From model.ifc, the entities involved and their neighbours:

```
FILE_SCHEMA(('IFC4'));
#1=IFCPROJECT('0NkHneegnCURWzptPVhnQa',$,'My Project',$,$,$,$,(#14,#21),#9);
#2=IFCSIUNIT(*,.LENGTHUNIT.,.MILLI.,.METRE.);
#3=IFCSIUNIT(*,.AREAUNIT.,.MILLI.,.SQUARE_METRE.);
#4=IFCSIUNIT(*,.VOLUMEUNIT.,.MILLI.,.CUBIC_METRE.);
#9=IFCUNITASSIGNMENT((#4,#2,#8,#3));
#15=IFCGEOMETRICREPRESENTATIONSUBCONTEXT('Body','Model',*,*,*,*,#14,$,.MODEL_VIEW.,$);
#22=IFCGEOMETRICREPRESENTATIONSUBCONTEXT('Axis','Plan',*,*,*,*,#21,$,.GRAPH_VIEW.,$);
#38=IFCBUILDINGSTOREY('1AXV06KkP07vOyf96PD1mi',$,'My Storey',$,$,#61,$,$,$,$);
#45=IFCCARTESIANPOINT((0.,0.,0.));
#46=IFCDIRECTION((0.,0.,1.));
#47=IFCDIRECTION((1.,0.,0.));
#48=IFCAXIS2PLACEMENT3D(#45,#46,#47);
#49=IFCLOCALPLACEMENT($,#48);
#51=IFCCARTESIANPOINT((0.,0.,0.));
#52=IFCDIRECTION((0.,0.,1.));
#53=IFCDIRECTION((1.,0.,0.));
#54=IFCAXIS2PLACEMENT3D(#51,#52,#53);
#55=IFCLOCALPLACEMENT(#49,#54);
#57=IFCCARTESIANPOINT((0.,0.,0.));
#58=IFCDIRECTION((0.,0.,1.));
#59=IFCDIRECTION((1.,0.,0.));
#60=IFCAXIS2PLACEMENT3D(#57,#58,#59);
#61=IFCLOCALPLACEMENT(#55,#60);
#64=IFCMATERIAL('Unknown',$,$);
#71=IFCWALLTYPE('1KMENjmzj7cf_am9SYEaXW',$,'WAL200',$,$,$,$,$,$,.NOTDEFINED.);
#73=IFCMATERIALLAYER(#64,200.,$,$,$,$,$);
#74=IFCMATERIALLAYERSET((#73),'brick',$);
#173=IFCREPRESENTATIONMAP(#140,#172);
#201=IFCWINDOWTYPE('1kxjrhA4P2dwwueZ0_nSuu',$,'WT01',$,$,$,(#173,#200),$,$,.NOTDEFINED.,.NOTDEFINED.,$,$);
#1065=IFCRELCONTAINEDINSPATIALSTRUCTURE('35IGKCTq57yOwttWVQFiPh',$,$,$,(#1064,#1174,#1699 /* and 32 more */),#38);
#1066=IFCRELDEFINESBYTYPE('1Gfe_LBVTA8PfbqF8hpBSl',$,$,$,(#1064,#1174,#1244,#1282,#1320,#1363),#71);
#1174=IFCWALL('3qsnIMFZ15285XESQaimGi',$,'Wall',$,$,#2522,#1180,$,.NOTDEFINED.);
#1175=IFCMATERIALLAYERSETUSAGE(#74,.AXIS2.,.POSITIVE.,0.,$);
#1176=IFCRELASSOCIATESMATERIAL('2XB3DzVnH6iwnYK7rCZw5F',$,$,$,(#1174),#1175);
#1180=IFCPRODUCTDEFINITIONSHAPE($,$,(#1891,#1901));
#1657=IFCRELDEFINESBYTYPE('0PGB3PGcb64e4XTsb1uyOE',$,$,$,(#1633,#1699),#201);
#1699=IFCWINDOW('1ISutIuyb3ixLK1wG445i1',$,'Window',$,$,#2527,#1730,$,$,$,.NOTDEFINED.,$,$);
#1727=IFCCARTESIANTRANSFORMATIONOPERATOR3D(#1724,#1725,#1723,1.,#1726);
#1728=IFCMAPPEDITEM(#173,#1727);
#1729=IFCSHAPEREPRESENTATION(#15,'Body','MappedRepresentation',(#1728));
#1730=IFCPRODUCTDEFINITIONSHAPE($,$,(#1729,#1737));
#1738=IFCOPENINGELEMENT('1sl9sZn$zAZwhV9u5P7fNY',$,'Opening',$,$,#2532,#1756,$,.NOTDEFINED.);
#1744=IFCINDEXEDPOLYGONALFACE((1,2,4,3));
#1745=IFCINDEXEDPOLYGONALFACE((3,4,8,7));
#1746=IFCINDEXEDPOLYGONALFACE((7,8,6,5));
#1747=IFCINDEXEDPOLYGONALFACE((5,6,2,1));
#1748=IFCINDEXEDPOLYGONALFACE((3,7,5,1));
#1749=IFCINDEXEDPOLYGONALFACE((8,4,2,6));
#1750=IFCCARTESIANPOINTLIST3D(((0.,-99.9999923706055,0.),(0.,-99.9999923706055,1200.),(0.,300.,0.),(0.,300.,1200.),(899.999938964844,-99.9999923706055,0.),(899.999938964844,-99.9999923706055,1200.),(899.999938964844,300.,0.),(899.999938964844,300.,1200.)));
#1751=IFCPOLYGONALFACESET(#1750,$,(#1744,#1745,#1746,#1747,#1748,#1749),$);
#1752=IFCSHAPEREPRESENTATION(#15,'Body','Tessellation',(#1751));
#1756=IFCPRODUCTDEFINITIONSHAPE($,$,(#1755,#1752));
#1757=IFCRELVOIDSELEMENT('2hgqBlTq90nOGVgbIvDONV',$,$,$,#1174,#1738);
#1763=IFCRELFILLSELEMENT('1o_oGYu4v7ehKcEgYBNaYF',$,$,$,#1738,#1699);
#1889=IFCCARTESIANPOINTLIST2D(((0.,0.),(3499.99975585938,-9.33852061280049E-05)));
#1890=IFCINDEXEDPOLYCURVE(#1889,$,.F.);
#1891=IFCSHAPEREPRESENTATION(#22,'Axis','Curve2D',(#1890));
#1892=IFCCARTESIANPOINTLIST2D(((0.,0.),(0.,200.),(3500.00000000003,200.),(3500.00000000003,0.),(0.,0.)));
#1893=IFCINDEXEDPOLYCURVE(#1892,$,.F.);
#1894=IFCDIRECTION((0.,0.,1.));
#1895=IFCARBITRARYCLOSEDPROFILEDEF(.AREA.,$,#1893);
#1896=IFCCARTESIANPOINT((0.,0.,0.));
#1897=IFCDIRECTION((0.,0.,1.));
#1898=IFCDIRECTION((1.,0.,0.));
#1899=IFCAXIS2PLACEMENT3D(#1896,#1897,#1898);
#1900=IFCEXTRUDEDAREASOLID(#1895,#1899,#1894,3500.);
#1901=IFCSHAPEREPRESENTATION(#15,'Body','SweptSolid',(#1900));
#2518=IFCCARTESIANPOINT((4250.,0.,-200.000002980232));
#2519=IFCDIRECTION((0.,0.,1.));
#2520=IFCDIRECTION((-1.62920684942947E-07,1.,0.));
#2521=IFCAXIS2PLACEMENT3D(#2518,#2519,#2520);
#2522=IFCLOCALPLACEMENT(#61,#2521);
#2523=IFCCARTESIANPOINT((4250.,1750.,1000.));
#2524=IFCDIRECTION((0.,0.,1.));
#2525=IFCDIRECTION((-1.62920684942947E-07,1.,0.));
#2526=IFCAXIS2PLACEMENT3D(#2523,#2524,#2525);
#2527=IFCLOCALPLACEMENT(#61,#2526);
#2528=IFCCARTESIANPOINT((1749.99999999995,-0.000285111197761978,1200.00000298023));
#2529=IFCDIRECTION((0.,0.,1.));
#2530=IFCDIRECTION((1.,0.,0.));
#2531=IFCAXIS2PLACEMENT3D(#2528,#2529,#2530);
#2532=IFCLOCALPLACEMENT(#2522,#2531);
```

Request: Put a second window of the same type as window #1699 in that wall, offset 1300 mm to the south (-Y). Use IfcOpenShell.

```python
import ifcopenshell
import ifcopenshell.api.feature
import ifcopenshell.api.geometry
import ifcopenshell.api.root
import ifcopenshell.geom
import ifcopenshell.util.element
import ifcopenshell.util.placement
import ifcopenshell.util.shape
import ifcopenshell.util.unit

model = ifcopenshell.open("model.ifc")
unit_scale = ifcopenshell.util.unit.calculate_unit_scale(model)
settings = ifcopenshell.geom.settings()


def volume(element):
    """Net volume in cubic metres, openings subtracted."""
    shape = ifcopenshell.geom.create_shape(settings, element)
    return ifcopenshell.util.shape.get_volume(shape.geometry)


window = model.by_id(1699)
opening = window.FillsVoids[0].RelatingOpeningElement
wall = opening.VoidsElements[0].RelatingBuildingElement
before = volume(wall)
shift = ifcopenshell.util.placement.get_local_placement(wall.ObjectPlacement)[:3, 0] * -1.3 / unit_scale

# copy_class copies the void relationship, type, container and properties, but no geometry.
new_opening = ifcopenshell.api.root.copy_class(model, product=opening)
new_opening.Representation = ifcopenshell.util.element.copy_deep(
    model, opening.Representation, exclude=["IfcGeometricRepresentationContext", "IfcRepresentationMap"]
)
new_window = ifcopenshell.api.root.copy_class(model, product=window)
new_window.Representation = ifcopenshell.util.element.copy_deep(
    model, window.Representation, exclude=["IfcGeometricRepresentationContext", "IfcRepresentationMap"]
)
ifcopenshell.api.feature.add_filling(model, opening=new_opening, element=new_window)

for old, new in ((opening, new_opening), (window, new_window)):
    matrix = ifcopenshell.util.placement.get_local_placement(old.ObjectPlacement)
    matrix[:3, 3] += shift
    ifcopenshell.api.geometry.edit_object_placement(model, product=new, matrix=matrix, is_si=False)

after = volume(wall)

print(f"wall volume {before:.3f} -> {after:.3f} m3")

model.write("model_updated.ifc")
```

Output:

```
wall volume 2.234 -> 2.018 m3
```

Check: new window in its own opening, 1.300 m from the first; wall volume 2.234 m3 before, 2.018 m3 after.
